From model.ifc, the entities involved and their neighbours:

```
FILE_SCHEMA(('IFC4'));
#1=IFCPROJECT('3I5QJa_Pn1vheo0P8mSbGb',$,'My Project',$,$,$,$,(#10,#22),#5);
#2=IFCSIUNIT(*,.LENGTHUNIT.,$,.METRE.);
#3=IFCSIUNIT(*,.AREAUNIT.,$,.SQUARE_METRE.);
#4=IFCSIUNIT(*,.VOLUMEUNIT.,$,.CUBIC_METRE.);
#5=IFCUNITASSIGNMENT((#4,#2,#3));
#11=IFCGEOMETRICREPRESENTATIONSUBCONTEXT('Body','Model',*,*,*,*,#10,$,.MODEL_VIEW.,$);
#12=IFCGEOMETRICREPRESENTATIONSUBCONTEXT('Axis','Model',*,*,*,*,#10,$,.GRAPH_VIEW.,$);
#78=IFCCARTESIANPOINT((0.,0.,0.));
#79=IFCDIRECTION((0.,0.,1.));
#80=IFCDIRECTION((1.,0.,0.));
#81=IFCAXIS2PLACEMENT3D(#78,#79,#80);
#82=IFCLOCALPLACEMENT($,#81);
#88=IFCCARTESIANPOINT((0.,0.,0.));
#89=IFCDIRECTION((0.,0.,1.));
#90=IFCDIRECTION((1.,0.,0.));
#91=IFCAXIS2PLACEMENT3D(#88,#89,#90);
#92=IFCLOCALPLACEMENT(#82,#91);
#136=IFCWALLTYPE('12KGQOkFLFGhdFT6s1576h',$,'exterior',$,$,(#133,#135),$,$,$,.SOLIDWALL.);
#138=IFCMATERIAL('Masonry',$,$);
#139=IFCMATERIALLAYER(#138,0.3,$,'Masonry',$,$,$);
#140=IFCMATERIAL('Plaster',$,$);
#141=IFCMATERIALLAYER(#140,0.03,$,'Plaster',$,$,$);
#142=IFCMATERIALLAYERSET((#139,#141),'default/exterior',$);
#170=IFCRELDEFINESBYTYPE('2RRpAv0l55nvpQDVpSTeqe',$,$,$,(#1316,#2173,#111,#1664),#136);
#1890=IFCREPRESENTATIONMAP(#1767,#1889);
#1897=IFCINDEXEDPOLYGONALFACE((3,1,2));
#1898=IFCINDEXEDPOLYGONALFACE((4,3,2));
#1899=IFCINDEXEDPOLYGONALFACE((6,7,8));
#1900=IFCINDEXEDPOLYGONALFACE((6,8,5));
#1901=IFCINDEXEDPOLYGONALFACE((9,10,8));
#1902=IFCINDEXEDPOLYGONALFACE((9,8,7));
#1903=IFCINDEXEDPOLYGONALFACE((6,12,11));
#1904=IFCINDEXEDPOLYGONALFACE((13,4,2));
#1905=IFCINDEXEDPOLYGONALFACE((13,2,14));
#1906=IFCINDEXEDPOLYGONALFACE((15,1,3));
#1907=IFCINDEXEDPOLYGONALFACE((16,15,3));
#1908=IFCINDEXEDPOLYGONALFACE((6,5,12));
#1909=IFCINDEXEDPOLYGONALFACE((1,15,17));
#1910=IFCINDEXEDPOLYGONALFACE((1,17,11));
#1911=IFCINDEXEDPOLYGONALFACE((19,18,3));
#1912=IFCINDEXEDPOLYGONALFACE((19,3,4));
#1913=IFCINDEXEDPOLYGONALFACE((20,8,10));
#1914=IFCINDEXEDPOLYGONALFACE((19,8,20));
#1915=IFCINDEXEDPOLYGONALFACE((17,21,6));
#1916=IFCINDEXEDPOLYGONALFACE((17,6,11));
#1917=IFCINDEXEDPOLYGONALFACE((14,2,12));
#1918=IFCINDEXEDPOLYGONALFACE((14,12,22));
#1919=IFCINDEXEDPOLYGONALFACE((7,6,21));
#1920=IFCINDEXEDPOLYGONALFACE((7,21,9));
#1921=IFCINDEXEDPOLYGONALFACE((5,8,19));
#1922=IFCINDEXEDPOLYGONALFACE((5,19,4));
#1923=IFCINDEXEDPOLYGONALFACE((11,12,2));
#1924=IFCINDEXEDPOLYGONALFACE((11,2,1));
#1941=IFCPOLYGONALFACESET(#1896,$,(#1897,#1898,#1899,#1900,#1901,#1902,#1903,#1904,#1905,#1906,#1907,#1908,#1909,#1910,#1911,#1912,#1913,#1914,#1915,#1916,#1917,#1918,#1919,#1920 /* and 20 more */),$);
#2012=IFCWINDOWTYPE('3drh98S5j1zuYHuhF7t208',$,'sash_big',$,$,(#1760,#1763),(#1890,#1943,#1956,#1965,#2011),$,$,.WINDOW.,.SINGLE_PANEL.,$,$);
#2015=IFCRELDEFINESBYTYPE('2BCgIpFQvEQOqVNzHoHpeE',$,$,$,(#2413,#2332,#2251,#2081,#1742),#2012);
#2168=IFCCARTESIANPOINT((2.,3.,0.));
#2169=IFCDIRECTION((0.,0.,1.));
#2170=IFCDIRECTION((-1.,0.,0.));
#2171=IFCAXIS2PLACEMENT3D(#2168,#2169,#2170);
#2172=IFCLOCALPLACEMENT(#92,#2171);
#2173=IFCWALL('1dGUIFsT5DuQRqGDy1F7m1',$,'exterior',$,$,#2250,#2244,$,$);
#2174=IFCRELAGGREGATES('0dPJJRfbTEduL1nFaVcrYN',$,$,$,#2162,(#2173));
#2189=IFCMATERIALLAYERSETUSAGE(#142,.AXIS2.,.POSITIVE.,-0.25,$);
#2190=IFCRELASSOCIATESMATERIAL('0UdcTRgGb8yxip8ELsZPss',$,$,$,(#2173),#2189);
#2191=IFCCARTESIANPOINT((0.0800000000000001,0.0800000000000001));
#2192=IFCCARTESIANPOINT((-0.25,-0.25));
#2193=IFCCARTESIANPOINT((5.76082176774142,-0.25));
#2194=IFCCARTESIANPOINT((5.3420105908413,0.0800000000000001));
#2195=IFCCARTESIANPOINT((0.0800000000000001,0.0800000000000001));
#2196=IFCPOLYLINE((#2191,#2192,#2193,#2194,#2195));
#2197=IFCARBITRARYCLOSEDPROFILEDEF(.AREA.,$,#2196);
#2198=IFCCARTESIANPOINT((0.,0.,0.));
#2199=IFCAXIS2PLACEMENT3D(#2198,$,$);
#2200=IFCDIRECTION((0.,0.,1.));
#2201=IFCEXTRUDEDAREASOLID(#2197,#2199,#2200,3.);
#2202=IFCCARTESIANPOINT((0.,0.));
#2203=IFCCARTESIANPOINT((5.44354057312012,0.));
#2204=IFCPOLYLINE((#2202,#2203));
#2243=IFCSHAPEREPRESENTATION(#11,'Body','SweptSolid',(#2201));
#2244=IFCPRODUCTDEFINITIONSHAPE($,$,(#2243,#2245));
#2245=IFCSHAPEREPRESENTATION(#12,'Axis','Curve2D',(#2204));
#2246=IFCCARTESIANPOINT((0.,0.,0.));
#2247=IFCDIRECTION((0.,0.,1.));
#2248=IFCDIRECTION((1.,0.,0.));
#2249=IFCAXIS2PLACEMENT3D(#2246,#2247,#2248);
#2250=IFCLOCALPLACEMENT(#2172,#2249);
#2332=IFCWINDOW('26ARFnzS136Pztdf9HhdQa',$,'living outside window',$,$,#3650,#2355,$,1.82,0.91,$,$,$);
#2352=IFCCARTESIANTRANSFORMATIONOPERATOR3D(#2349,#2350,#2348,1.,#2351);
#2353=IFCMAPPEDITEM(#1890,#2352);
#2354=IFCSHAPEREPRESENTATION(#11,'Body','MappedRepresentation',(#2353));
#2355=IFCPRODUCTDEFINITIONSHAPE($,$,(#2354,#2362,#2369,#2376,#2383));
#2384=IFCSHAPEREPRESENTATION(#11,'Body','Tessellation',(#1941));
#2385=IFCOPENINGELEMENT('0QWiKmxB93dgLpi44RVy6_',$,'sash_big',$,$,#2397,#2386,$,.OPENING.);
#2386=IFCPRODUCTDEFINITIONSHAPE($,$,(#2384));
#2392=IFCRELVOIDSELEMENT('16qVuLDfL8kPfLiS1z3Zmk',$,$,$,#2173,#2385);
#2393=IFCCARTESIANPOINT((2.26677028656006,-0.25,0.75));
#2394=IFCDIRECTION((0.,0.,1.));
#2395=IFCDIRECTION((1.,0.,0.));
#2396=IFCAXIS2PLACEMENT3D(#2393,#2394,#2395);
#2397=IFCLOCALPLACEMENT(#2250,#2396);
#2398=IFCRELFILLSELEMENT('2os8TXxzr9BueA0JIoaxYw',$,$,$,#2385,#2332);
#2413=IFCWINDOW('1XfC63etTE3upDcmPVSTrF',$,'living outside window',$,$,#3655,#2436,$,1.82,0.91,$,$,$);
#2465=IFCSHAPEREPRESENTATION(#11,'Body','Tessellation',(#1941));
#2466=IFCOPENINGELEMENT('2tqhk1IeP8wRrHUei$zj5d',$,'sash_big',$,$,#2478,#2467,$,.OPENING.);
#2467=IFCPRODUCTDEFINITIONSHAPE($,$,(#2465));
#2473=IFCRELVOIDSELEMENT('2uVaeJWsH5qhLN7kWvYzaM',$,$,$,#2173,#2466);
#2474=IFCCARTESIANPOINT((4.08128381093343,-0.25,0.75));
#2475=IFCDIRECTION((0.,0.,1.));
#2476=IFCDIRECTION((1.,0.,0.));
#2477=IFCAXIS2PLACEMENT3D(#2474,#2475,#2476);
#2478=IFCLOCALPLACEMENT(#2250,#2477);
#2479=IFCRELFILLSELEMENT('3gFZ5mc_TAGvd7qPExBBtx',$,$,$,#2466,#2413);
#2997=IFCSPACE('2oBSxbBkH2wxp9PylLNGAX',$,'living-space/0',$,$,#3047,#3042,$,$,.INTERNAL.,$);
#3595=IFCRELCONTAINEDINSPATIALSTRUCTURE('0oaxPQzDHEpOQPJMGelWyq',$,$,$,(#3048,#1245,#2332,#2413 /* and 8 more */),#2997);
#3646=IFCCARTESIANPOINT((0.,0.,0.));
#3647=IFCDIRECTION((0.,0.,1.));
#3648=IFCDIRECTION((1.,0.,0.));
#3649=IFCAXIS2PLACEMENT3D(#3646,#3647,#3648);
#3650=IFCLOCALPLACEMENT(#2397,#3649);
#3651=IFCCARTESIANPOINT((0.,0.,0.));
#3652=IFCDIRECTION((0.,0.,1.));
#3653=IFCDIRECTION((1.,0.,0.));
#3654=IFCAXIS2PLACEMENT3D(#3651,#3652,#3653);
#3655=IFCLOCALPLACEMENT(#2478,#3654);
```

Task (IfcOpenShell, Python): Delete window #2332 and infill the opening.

```python
import ifcopenshell
import ifcopenshell.api.feature
import ifcopenshell.api.root
import ifcopenshell.geom
import ifcopenshell.util.shape

model = ifcopenshell.open("model.ifc")
settings = ifcopenshell.geom.settings()


def volume(element):
    """Net volume in cubic metres, openings subtracted."""
    shape = ifcopenshell.geom.create_shape(settings, element)
    return ifcopenshell.util.shape.get_volume(shape.geometry)


window = model.by_guid("26ARFnzS136Pztdf9HhdQa")
opening = window.FillsVoids[0].RelatingOpeningElement
wall = opening.VoidsElements[0].RelatingBuildingElement
before = volume(wall)

ifcopenshell.api.root.remove_product(model, product=window)
ifcopenshell.api.feature.remove_feature(model, feature=opening)

after = volume(wall)

print(f"wall volume {before:.3f} -> {after:.3f} m3")

model.write("model_v2.ifc")
```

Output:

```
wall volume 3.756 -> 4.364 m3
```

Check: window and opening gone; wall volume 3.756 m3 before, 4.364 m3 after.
